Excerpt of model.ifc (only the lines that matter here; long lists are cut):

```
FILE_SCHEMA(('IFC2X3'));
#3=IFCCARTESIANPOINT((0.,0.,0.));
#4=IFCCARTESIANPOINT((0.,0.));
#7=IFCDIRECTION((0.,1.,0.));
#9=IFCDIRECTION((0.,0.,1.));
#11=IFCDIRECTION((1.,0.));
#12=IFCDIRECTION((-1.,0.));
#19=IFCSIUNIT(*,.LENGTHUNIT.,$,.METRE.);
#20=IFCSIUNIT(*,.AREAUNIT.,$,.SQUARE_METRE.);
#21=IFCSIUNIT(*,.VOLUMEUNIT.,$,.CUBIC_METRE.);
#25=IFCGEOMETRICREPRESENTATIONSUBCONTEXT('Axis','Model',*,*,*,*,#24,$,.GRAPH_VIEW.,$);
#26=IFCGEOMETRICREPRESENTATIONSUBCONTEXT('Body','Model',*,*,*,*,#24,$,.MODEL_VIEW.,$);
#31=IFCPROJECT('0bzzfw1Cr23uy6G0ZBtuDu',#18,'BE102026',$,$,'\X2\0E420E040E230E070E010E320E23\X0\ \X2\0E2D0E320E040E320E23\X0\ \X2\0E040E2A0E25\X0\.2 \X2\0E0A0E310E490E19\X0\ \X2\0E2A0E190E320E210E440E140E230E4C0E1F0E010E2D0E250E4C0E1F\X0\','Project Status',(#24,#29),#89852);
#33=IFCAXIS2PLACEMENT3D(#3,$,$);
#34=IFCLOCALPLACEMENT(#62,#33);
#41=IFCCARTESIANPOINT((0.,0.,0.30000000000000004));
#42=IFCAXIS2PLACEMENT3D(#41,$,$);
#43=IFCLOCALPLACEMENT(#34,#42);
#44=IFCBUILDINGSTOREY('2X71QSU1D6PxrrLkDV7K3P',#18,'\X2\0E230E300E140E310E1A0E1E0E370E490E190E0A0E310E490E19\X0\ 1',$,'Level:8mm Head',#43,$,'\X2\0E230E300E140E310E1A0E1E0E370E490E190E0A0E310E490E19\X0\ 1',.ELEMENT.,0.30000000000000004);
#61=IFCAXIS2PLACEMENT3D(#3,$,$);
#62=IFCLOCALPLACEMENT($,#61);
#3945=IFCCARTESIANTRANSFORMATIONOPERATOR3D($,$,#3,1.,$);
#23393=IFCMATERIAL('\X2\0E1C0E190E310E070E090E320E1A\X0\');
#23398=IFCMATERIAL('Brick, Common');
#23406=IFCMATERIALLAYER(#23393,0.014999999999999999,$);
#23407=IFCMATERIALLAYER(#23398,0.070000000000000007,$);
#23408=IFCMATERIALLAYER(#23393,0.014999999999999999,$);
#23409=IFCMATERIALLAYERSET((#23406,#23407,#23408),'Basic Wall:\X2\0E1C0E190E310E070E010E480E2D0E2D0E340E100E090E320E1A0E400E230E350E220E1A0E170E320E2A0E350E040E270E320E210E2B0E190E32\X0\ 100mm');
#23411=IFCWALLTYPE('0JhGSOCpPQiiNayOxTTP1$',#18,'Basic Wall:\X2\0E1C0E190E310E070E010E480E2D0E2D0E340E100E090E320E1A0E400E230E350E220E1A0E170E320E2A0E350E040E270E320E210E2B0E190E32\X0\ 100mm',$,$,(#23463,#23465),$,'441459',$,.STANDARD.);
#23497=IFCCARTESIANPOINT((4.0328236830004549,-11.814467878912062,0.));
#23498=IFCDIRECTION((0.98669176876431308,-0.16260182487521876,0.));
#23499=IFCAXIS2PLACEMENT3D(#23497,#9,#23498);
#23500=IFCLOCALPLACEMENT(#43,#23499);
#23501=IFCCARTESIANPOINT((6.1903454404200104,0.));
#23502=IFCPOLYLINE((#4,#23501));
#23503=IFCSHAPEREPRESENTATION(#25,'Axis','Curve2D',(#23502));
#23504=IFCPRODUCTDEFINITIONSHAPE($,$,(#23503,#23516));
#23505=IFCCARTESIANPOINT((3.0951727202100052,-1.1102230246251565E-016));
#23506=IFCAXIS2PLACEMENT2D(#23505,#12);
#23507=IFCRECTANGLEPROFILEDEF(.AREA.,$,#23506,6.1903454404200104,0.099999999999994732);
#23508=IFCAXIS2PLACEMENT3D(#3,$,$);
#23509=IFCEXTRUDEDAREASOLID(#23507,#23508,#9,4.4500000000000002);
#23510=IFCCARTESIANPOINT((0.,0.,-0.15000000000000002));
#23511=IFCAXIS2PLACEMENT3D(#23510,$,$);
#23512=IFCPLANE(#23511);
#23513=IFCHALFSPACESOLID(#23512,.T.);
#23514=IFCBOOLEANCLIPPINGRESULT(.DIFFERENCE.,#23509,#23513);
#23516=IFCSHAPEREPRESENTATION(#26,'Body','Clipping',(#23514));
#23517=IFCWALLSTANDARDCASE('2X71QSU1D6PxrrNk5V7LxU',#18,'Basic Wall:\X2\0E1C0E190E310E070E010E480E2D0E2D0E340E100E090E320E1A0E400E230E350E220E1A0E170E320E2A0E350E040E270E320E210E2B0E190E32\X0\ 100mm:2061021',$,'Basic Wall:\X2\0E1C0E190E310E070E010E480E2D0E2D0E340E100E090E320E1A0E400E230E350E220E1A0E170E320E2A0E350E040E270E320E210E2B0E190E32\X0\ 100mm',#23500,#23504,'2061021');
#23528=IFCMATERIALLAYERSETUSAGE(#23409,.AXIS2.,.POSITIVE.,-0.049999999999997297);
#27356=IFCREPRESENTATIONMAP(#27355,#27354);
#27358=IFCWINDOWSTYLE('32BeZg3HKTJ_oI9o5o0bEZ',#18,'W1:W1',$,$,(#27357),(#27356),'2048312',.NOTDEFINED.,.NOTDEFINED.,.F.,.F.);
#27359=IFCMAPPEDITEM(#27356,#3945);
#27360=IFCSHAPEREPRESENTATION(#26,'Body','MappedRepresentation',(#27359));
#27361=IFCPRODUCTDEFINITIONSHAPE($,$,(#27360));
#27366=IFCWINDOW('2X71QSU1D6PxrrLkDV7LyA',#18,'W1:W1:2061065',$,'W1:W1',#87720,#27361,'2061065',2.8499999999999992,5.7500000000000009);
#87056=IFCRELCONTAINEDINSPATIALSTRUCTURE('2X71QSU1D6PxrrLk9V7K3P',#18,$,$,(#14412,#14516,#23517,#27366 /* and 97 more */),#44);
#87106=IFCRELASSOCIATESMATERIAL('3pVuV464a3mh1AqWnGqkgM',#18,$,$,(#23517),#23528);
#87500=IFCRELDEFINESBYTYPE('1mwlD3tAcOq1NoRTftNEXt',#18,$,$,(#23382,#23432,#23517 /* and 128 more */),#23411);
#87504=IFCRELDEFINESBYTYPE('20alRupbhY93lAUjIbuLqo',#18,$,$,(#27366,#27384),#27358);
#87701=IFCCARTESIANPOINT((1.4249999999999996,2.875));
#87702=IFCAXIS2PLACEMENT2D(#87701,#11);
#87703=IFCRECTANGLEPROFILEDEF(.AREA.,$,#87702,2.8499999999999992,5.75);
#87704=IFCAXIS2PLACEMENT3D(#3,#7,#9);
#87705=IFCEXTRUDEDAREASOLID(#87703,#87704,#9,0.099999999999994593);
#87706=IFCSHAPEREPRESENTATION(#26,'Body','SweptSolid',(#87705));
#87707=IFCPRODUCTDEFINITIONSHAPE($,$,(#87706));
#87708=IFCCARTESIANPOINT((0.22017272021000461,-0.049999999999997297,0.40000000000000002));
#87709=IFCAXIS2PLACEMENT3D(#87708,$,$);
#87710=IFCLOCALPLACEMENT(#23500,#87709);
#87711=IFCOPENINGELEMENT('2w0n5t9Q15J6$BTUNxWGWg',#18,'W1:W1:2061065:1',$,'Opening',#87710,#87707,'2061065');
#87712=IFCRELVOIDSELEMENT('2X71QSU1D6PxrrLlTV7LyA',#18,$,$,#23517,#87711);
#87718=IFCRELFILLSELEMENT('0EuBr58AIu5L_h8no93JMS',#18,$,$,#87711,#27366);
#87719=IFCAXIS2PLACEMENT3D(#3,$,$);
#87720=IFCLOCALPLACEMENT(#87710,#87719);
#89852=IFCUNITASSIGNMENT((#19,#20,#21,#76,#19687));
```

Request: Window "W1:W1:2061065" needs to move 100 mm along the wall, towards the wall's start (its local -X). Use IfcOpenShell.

```python
import ifcopenshell
import ifcopenshell.api.geometry
import ifcopenshell.util.placement
import ifcopenshell.util.unit

model = ifcopenshell.open("model.ifc")
unit_scale = ifcopenshell.util.unit.calculate_unit_scale(model)

window = model.by_guid("2X71QSU1D6PxrrLkDV7LyA")
opening = window.FillsVoids[0].RelatingOpeningElement
wall = opening.VoidsElements[0].RelatingBuildingElement

wall_matrix = ifcopenshell.util.placement.get_local_placement(wall.ObjectPlacement)
shift = wall_matrix[:3, 0] * -0.1 / unit_scale
before = ifcopenshell.util.placement.get_local_placement(window.ObjectPlacement)[:3, 3].copy()

# The window is placed relative to its opening, so it follows when the opening moves.
matrix = ifcopenshell.util.placement.get_local_placement(opening.ObjectPlacement)
matrix[:3, 3] += shift
ifcopenshell.api.geometry.edit_object_placement(
    model, product=opening, matrix=matrix, is_si=False, should_transform_children=True
)

after = ifcopenshell.util.placement.get_local_placement(window.ObjectPlacement)[:3, 3]
print("window moved by", (after - before).round(3) + 0.0)

model.write("model_rev.ifc")
```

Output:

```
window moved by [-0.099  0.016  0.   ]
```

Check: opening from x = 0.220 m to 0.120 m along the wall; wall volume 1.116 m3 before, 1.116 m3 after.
